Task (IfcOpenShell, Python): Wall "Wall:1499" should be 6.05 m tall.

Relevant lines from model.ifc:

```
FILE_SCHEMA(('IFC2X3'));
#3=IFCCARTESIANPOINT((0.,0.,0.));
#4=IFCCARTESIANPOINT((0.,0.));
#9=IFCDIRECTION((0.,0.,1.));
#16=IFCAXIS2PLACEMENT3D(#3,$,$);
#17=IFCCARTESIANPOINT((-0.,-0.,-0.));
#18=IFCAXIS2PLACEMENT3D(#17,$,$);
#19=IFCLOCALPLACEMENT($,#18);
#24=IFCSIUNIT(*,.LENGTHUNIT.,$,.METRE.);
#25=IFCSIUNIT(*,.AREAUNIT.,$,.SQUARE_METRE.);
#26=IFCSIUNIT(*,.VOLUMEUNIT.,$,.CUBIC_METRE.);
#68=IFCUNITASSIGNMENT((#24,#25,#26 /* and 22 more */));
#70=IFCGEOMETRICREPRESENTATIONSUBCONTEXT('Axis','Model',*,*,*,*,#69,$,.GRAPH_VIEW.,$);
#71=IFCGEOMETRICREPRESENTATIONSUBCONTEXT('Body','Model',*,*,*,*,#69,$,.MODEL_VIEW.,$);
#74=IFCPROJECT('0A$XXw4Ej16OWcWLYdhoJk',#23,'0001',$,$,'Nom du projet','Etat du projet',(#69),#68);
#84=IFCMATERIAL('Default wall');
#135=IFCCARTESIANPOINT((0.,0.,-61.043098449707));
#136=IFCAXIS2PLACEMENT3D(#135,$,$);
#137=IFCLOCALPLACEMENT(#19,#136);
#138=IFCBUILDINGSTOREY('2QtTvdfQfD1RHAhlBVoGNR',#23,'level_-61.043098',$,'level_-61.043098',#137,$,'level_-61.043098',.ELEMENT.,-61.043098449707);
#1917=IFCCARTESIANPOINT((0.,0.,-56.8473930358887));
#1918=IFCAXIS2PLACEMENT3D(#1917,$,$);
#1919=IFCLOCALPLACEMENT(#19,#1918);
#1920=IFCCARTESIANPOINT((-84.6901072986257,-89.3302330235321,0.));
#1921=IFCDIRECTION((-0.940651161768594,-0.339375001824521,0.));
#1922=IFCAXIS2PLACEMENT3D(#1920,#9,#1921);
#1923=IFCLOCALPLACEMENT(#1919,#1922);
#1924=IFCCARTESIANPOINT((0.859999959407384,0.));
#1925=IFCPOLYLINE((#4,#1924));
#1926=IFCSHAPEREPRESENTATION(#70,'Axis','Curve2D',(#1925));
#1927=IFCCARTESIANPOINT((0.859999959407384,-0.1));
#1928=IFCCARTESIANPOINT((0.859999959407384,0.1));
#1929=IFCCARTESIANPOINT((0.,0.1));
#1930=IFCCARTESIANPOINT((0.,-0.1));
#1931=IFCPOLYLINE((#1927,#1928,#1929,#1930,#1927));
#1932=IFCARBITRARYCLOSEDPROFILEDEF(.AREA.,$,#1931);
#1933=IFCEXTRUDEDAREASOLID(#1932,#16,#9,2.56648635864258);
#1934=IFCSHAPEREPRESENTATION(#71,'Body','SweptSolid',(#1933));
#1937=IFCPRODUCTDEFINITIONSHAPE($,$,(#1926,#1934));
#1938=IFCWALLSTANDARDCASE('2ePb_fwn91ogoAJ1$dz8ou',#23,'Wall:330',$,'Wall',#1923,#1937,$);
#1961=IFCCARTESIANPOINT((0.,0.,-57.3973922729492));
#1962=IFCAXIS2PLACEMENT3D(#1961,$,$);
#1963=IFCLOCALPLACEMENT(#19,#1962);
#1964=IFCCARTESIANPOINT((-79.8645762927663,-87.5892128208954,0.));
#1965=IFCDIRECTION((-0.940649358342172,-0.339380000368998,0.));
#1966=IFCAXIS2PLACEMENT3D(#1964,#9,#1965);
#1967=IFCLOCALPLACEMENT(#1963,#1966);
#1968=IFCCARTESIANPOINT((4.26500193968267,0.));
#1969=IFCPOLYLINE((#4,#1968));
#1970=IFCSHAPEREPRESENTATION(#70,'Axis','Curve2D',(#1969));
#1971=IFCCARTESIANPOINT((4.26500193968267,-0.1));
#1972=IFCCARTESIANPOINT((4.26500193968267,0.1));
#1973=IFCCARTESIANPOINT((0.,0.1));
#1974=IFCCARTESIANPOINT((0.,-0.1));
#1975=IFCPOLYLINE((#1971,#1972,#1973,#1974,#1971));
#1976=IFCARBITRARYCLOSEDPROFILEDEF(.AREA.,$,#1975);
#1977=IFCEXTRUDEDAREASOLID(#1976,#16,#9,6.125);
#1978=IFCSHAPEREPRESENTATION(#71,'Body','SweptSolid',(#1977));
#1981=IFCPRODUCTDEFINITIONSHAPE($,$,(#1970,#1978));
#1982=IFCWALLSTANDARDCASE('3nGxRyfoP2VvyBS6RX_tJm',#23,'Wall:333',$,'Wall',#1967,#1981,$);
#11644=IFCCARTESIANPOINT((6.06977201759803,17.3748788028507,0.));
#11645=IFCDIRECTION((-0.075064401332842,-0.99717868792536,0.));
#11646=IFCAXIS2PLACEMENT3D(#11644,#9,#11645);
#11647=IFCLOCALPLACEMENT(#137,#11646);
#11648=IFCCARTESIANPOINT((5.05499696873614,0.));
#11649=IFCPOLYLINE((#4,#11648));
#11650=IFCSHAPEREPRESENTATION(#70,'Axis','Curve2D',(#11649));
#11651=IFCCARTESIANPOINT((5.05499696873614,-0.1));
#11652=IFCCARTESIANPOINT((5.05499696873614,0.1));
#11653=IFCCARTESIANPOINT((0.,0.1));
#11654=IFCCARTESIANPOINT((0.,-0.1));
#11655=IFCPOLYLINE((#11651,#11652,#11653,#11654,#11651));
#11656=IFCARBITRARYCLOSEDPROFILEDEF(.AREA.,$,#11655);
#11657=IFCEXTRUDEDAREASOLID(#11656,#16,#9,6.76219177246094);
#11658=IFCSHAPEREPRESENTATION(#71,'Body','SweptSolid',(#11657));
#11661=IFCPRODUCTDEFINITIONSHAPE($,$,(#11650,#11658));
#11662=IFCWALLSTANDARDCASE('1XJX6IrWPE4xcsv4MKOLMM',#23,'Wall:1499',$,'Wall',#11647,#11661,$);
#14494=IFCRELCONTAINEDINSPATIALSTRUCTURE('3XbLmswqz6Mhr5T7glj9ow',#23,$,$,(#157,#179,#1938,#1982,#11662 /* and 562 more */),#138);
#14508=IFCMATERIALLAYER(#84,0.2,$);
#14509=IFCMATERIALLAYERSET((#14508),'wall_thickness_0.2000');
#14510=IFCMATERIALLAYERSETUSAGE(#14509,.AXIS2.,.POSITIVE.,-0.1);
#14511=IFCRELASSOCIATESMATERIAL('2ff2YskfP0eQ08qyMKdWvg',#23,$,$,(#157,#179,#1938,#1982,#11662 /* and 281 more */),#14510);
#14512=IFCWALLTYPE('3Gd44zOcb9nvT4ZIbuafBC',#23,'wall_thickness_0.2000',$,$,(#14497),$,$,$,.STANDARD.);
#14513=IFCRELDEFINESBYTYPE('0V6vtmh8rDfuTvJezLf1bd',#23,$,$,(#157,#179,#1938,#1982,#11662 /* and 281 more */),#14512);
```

```python
import ifcopenshell
import ifcopenshell.geom
import ifcopenshell.util.representation
import ifcopenshell.util.shape
import ifcopenshell.util.unit

model = ifcopenshell.open("model.ifc")
unit_scale = ifcopenshell.util.unit.calculate_unit_scale(model)
settings = ifcopenshell.geom.settings()


def volume(element):
    """Net volume in cubic metres, openings subtracted."""
    shape = ifcopenshell.geom.create_shape(settings, element)
    return ifcopenshell.util.shape.get_volume(shape.geometry)


wall = model.by_id(11662)
before = volume(wall)

body = ifcopenshell.util.representation.get_representation(wall, "Model", "Body")
solid = body.Items[0]
old_height = solid.Depth
solid.Depth = 6.05 / unit_scale
after = volume(wall)

print(f"height {old_height:g} -> {solid.Depth:g}, volume {before:.3f} -> {after:.3f} m3")

model.write("model_v2.ifc")
```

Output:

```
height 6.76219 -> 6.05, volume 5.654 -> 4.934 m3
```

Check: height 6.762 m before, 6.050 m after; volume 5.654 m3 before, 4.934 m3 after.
